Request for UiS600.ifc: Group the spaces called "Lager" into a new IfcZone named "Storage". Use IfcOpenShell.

First a look at what the model holds.

```python
import ifcopenshell

model = ifcopenshell.open("UiS600.ifc")
print(model.schema)
seen = {}
for space in model.by_type("IfcSpace"):
    seen[space.LongName] = seen.get(space.LongName, 0) + 1
for name, count in sorted(seen.items(), key=str):
    print(count, "x", name)
print("zones:", [z.Name for z in model.by_type("IfcZone")][:20])
```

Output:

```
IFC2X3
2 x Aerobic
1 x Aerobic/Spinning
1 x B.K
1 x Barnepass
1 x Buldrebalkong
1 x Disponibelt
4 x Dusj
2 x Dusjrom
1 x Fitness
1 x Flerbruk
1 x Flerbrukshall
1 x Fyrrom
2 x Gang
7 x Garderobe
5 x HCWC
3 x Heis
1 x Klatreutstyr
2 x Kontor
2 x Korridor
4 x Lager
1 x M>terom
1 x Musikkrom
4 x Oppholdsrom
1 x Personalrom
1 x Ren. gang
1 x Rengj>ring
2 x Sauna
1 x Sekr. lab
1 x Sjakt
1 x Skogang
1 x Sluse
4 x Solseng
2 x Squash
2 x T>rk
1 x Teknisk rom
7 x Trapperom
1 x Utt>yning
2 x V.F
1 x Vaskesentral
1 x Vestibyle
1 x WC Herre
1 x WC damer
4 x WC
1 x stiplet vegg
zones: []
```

```python
import ifcopenshell
import ifcopenshell.api.group
import ifcopenshell.api.root

model = ifcopenshell.open("UiS600.ifc")

names = {"Lager"}
spaces = [s for s in model.by_type("IfcSpace") if s.LongName in names]

zone = ifcopenshell.api.root.create_entity(model, ifc_class="IfcZone", name="Storage")
ifcopenshell.api.group.assign_group(model, products=spaces, group=zone)
print(len(spaces), "spaces in", zone.Name)

model.write("UiS600_edited.ifc")
```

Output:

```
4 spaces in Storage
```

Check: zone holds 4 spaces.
